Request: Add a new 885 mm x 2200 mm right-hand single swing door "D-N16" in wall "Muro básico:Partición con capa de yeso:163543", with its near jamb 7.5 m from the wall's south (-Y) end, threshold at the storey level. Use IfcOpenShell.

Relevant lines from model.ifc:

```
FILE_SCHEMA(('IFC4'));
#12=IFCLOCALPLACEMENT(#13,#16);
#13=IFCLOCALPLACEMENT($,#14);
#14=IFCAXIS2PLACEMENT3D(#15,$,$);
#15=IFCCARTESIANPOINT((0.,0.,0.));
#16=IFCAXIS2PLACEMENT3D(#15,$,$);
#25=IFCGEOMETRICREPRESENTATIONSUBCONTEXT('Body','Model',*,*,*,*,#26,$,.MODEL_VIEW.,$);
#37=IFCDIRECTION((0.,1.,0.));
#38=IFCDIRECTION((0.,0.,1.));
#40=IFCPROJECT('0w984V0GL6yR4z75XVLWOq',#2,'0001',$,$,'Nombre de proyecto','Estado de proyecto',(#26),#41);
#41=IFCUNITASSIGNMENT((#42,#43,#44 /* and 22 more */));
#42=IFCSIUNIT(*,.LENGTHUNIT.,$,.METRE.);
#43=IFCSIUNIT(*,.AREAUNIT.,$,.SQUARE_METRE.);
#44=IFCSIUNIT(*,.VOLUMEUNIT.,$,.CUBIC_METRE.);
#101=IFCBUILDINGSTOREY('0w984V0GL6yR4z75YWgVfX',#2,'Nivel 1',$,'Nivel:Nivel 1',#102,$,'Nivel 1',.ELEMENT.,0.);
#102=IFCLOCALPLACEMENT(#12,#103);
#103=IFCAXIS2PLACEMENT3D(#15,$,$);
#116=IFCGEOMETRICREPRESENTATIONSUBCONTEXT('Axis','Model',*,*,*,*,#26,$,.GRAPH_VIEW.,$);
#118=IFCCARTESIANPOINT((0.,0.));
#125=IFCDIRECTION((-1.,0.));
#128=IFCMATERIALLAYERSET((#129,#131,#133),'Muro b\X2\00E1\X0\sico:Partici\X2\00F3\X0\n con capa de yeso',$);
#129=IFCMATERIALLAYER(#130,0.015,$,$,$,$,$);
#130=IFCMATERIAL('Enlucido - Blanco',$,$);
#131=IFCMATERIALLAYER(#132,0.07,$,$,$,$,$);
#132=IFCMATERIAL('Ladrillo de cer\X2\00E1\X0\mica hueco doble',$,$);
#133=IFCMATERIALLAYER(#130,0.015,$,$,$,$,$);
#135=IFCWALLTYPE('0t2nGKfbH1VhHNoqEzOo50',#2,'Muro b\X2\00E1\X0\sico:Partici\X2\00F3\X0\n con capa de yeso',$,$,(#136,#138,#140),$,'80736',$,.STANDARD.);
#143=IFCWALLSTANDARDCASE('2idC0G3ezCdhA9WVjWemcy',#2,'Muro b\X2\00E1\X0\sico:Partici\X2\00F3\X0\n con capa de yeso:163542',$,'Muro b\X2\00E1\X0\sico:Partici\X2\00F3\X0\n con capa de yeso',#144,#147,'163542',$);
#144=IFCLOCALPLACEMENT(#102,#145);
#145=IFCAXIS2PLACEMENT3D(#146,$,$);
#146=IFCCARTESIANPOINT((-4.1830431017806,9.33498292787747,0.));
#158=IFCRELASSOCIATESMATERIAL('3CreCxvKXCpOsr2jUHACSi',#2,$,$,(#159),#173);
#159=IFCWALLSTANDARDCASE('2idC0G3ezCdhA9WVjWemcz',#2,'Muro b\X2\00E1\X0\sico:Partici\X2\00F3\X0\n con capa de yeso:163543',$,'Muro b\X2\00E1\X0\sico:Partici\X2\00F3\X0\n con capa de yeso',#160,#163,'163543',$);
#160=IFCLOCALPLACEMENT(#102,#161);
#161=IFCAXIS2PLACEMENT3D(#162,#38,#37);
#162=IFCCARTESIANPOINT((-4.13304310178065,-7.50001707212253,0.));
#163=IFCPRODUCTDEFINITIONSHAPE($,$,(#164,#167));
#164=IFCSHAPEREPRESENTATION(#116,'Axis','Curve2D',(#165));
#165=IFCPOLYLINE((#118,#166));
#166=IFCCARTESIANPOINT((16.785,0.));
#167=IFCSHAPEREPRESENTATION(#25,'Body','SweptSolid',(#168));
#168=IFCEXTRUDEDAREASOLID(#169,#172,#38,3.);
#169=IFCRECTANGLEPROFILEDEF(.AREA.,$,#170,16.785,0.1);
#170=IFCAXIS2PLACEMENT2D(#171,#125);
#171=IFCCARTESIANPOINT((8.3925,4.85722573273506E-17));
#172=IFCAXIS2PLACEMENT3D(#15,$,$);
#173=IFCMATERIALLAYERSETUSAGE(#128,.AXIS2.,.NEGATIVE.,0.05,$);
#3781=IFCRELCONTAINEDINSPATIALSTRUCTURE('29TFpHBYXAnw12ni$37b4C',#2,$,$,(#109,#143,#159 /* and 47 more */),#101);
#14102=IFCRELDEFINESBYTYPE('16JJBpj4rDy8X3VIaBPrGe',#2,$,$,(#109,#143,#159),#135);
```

```python
import numpy as np
import ifcopenshell
import ifcopenshell.api.feature
import ifcopenshell.api.geometry
import ifcopenshell.api.root
import ifcopenshell.api.spatial
import ifcopenshell.geom
import ifcopenshell.util.element
import ifcopenshell.util.placement
import ifcopenshell.util.representation
import ifcopenshell.util.shape
import ifcopenshell.util.unit

model = ifcopenshell.open("model.ifc")
unit_scale = ifcopenshell.util.unit.calculate_unit_scale(model)
settings = ifcopenshell.geom.settings()


def volume(element):
    """Net volume in cubic metres, openings subtracted."""
    shape = ifcopenshell.geom.create_shape(settings, element)
    return ifcopenshell.util.shape.get_volume(shape.geometry)


wall = model.by_guid("2idC0G3ezCdhA9WVjWemcz")
storey = ifcopenshell.util.element.get_container(wall, ifc_class="IfcBuildingStorey")
context = ifcopenshell.util.representation.get_context(model, "Model", "Body", "MODEL_VIEW")
before = volume(wall)

width, height, from_end, sill = 0.885, 2.2, 7.5, 0.0  # metres

# The wall runs along its own X axis, and the end named is its -X end.
wall_shape = ifcopenshell.geom.create_shape(settings, wall)
x, y, z = ifcopenshell.util.shape.get_vertices(wall_shape.geometry).T
start = x.min() + from_end
face, thickness = float(y.min()), float(y.max() - y.min())
wall_matrix = ifcopenshell.util.placement.get_local_placement(wall.ObjectPlacement)
level = ifcopenshell.util.placement.get_local_placement(storey.ObjectPlacement)[2, 3]


def in_wall(x, y):
    """Placement at x, y metres in the wall's axes, at sill height."""
    matrix = wall_matrix.copy()
    matrix[:, 3] = wall_matrix @ np.array([x / unit_scale, y / unit_scale, 0.0, 1.0])
    matrix[2, 3] = level + sill / unit_scale
    return matrix


# Opening: a box that overshoots both wall faces by 50 mm.
opening = ifcopenshell.api.root.create_entity(model, ifc_class="IfcOpeningElement", predefined_type="OPENING")
box = ifcopenshell.api.geometry.add_wall_representation(
    model, context=context, length=width, height=height, thickness=thickness + 0.1
)
ifcopenshell.api.geometry.assign_representation(model, product=opening, representation=box)
ifcopenshell.api.geometry.edit_object_placement(model, product=opening, matrix=in_wall(start, face - 0.05), is_si=False)
ifcopenshell.api.feature.add_feature(model, feature=opening, element=wall)

door = ifcopenshell.api.root.create_entity(model, ifc_class="IfcDoor", name="D-N16", predefined_type="DOOR")
door.OverallWidth, door.OverallHeight = width / unit_scale, height / unit_scale
door.OperationType = "SINGLE_SWING_RIGHT"
body = ifcopenshell.api.geometry.add_door_representation(
    model,
    context=context,
    overall_width=door.OverallWidth,
    overall_height=door.OverallHeight,
    operation_type="SINGLE_SWING_RIGHT",
    lining_properties={"LiningDepth": thickness / unit_scale, "ThresholdDepth": thickness / unit_scale},
)
ifcopenshell.api.geometry.assign_representation(model, product=door, representation=body)
ifcopenshell.api.spatial.assign_container(model, products=[door], relating_structure=storey)
ifcopenshell.api.feature.add_filling(model, opening=opening, element=door)

# The lining spans the wall, so the door starts at the wall face.
ifcopenshell.api.geometry.edit_object_placement(model, product=door, matrix=in_wall(start, face), is_si=False)

after = volume(wall)

print(f"wall volume {before:.3f} -> {after:.3f} m3")

model.write("model_updated.ifc")
```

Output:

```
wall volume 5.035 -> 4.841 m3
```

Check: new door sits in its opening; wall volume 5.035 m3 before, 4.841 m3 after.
